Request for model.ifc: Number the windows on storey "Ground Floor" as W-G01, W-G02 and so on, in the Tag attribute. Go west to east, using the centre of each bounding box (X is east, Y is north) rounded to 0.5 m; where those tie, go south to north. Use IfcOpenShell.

First a look at what the model holds.

```python
import ifcopenshell
import ifcopenshell.util.element
import ifcopenshell.util.placement

model = ifcopenshell.open("model.ifc")
print(model.schema)
storey = next(s for s in model.by_type("IfcBuildingStorey") if s.Name == "Ground Floor")
windows = [e for e in ifcopenshell.util.element.get_decomposition(storey) if e.is_a("IfcWindow")]
for e in sorted(windows, key=lambda e: e.id()):
    origin = ifcopenshell.util.placement.get_local_placement(e.ObjectPlacement)[:3, 3]
    print(e.id(), e.Tag, e.Name, origin.round(2) + 0.0, sep=" | ")
```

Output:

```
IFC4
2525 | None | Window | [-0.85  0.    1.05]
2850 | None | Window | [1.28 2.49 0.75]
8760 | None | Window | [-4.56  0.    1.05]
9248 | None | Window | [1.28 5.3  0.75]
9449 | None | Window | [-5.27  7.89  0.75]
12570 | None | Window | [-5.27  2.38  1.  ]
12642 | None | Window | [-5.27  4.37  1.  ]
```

```python
import ifcopenshell
import ifcopenshell.geom
import ifcopenshell.util.element
import ifcopenshell.util.shape

model = ifcopenshell.open("model.ifc")
settings = ifcopenshell.geom.settings()
settings.set("use-world-coords", True)


def centre(element):
    shape = ifcopenshell.geom.create_shape(settings, element)
    return ifcopenshell.util.shape.get_bbox_centroid(shape.geometry)


storey = next(s for s in model.by_type("IfcBuildingStorey") if s.Name == "Ground Floor")
windows = [e for e in ifcopenshell.util.element.get_decomposition(storey) if e.is_a("IfcWindow")]

# Insertion points can sit at a corner or the storey origin, so sort by the geometry (in metres).
centres = {e: centre(e) for e in windows}
windows.sort(key=lambda e: (round(centres[e][0] / 0.5), centres[e][1]))

for i, e in enumerate(windows, start=1):
    number = f"W-G{i:02d}"
    e.Tag = number
    print(e.id(), number)

model.write("model-out.ifc")
```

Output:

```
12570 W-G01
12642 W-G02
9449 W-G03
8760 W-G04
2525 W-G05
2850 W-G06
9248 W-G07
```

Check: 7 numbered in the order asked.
